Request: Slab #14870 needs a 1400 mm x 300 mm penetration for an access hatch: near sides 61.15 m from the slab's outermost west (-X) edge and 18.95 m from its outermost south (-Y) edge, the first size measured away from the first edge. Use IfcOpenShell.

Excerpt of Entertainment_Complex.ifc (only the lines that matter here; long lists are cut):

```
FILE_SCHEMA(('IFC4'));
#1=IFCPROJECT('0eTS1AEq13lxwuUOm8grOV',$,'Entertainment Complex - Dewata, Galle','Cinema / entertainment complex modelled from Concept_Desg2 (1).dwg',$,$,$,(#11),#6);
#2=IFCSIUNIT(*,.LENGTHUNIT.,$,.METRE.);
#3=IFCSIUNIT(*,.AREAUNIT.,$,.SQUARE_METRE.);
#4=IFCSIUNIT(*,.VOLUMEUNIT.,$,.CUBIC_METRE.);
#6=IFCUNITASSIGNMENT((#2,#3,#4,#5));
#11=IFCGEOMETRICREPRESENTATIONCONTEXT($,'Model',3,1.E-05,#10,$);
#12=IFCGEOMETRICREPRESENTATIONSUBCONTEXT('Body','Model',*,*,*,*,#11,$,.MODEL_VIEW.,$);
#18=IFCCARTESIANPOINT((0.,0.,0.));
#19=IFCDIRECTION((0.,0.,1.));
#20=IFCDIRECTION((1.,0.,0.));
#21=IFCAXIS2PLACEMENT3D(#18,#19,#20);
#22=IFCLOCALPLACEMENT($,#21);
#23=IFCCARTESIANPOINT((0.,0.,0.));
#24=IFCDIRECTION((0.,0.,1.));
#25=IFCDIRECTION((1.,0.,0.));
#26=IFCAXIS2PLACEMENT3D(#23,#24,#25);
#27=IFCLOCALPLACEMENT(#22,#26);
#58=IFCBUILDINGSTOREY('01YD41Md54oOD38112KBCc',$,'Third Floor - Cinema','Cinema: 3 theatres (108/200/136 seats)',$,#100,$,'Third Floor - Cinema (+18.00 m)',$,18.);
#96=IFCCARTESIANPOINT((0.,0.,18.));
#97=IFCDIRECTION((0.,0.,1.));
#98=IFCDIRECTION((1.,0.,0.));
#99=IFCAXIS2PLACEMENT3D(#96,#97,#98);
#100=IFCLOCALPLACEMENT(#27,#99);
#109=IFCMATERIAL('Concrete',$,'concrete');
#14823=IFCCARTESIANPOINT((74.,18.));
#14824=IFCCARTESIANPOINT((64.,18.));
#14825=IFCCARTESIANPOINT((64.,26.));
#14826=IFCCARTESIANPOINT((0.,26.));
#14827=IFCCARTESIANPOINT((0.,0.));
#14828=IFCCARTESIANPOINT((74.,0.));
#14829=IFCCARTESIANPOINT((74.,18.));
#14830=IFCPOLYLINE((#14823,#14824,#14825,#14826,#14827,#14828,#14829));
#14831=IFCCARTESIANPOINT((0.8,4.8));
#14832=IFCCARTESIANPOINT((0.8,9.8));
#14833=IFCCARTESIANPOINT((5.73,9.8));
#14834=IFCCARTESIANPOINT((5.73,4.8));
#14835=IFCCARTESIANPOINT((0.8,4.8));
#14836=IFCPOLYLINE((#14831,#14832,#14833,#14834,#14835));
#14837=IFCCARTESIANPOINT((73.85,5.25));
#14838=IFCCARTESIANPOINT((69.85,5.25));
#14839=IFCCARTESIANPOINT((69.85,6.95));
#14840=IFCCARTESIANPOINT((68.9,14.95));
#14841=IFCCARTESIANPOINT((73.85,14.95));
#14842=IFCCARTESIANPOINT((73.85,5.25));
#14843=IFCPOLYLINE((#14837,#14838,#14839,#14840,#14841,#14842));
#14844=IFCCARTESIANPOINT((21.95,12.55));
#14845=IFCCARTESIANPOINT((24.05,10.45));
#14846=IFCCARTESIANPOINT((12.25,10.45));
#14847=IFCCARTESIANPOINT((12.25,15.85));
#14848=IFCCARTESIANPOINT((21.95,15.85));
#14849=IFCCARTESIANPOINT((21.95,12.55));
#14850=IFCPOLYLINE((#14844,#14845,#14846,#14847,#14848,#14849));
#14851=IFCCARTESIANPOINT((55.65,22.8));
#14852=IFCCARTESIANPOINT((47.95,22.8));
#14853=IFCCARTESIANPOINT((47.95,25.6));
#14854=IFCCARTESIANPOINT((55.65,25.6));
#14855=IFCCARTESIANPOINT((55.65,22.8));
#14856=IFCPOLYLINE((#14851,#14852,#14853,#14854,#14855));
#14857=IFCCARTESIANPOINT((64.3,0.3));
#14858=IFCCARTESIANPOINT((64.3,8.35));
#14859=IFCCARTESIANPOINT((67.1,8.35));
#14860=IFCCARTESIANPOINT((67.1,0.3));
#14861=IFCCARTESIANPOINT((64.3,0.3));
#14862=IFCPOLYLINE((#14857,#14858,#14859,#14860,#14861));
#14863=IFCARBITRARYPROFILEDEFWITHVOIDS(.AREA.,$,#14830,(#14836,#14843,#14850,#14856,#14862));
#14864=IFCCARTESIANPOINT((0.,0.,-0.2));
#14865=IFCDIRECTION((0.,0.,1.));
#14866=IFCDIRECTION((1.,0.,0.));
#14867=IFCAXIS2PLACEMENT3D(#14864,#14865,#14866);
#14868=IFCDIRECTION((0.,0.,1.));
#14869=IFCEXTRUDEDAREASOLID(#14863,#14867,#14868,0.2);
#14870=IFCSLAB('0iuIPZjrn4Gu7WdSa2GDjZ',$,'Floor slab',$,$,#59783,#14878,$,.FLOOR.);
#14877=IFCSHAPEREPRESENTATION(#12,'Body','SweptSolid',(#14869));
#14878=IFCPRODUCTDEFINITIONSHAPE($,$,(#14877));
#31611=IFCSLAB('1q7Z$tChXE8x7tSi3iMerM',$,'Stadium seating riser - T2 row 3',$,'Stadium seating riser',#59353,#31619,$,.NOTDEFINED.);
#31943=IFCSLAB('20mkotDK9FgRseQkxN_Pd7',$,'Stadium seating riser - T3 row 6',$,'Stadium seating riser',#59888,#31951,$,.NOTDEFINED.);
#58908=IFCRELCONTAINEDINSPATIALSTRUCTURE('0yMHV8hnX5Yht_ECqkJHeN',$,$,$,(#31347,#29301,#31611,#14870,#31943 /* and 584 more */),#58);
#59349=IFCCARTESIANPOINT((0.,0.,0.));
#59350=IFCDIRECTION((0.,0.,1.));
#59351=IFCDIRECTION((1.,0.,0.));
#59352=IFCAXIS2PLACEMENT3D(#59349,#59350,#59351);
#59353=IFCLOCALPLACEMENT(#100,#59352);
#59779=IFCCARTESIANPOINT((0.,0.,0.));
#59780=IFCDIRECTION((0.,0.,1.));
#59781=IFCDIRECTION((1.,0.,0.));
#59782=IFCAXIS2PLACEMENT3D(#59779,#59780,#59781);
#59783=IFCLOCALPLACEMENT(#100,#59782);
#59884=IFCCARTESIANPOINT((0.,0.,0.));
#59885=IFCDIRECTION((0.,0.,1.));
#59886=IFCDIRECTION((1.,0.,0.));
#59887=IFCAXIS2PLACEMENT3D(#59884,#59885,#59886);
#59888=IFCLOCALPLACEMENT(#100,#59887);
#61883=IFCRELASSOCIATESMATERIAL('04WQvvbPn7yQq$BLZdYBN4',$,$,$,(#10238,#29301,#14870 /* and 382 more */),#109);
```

```python
import numpy as np
import ifcopenshell
import ifcopenshell.api.feature
import ifcopenshell.api.geometry
import ifcopenshell.api.root
import ifcopenshell.geom
import ifcopenshell.util.placement
import ifcopenshell.util.representation
import ifcopenshell.util.shape
import ifcopenshell.util.unit

model = ifcopenshell.open("Entertainment_Complex.ifc")
unit_scale = ifcopenshell.util.unit.calculate_unit_scale(model)
settings = ifcopenshell.geom.settings()


def volume(element):
    """Net volume in cubic metres, openings subtracted."""
    shape = ifcopenshell.geom.create_shape(settings, element)
    return ifcopenshell.util.shape.get_volume(shape.geometry)


slab = model.by_id(14870)
before = volume(slab)

# Extent in the slab's own axes, in metres. The edges named are its -X and -Y sides.
slab_shape = ifcopenshell.geom.create_shape(settings, slab)
vertices = ifcopenshell.util.shape.get_vertices(slab_shape.geometry)
x_min, y_min, bottom = vertices.min(axis=0)
top = vertices[:, 2].max()

opening = ifcopenshell.api.root.create_entity(model, ifc_class="IfcOpeningElement", name="Access hatch opening", predefined_type="OPENING")
context = ifcopenshell.util.representation.get_context(model, "Model", "Body", "MODEL_VIEW")
width, depth = 1.4, 0.3
outline = [(0.0, 0.0), (width, 0.0), (width, depth), (0.0, depth), (0.0, 0.0)]
# Overshoot both faces by 50 mm so the cut is clean.
shape = ifcopenshell.api.geometry.add_slab_representation(
    model, context=context, depth=top - bottom + 0.1, polyline=outline
)
ifcopenshell.api.geometry.assign_representation(model, product=opening, representation=shape)

matrix = ifcopenshell.util.placement.get_local_placement(slab.ObjectPlacement)
matrix[:, 3] = matrix @ np.append(np.array([x_min + 61.15, y_min + 18.95, bottom - 0.05]) / unit_scale, 1.0)
ifcopenshell.api.geometry.edit_object_placement(model, product=opening, matrix=matrix, is_si=False)
ifcopenshell.api.feature.add_feature(model, feature=opening, element=slab)

after = volume(slab)

print(f"slab volume {before:.3f} -> {after:.3f} m3")

model.write("Entertainment_Complex-out.ifc")
```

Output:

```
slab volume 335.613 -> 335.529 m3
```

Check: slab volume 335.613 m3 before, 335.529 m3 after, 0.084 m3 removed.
